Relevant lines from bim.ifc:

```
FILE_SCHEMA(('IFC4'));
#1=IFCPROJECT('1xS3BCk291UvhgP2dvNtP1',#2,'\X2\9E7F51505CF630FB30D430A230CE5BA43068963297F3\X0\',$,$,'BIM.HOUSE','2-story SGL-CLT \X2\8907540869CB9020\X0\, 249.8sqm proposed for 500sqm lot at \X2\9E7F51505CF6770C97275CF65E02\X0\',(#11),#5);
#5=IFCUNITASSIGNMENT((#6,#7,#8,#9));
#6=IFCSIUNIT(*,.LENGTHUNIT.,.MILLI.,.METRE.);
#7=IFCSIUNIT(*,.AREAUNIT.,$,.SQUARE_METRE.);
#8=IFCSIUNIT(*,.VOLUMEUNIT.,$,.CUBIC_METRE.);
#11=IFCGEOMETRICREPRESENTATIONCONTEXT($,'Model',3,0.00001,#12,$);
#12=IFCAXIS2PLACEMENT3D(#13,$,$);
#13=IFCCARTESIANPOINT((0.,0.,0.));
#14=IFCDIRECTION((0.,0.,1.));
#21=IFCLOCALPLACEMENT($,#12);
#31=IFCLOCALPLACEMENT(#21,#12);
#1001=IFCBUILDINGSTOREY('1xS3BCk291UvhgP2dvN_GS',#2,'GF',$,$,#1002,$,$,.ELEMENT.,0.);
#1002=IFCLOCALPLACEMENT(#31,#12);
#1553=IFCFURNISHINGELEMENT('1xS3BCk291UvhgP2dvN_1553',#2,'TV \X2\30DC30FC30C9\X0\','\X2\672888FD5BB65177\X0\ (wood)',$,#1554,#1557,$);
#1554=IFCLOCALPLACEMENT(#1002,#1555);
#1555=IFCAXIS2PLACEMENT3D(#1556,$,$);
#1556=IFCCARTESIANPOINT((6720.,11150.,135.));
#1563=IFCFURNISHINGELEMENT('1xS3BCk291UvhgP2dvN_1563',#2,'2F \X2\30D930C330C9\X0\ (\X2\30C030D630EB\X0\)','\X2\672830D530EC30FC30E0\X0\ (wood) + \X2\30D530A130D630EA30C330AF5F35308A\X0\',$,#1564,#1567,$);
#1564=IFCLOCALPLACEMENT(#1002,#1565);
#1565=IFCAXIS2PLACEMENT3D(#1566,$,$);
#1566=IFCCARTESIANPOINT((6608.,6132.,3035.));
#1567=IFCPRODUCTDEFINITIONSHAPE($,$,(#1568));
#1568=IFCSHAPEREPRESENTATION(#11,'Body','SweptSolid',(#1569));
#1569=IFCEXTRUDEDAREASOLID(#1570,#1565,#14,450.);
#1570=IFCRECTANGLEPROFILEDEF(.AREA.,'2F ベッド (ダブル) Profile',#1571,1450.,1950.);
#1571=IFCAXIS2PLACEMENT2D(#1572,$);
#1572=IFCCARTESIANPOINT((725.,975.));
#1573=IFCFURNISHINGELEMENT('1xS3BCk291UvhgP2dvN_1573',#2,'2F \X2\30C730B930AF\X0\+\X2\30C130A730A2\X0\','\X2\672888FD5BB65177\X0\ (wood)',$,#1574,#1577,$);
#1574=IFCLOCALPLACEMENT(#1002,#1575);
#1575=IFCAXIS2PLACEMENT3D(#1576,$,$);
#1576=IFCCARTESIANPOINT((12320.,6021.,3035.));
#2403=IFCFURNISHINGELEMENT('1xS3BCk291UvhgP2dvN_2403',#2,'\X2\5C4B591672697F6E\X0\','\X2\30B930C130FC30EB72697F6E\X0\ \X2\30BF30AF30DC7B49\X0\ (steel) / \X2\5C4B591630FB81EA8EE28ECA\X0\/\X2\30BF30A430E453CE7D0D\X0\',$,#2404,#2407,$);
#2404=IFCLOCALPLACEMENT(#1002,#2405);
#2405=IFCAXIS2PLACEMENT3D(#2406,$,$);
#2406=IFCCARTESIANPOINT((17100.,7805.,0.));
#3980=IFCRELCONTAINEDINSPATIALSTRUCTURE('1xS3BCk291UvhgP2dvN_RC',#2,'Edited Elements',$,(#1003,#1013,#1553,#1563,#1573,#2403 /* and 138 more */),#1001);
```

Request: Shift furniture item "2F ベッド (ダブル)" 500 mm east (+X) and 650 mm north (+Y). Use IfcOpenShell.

```python
import ifcopenshell
import ifcopenshell.api.geometry
import ifcopenshell.util.placement

model = ifcopenshell.open("bim.ifc")

item = model.by_guid("1xS3BCk291UvhgP2dvN_1563")
matrix = ifcopenshell.util.placement.get_local_placement(item.ObjectPlacement)
matrix[0, 3] += 500.0
matrix[1, 3] += 650.0
ifcopenshell.api.geometry.edit_object_placement(model, product=item, matrix=matrix, is_si=False)

print(ifcopenshell.util.placement.get_local_placement(item.ObjectPlacement).round(3) + 0.0)

model.write("bim_updated.ifc")
```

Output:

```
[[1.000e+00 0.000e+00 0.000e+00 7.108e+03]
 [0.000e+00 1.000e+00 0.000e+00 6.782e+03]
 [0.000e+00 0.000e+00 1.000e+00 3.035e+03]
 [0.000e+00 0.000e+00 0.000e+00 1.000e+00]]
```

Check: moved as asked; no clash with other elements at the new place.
